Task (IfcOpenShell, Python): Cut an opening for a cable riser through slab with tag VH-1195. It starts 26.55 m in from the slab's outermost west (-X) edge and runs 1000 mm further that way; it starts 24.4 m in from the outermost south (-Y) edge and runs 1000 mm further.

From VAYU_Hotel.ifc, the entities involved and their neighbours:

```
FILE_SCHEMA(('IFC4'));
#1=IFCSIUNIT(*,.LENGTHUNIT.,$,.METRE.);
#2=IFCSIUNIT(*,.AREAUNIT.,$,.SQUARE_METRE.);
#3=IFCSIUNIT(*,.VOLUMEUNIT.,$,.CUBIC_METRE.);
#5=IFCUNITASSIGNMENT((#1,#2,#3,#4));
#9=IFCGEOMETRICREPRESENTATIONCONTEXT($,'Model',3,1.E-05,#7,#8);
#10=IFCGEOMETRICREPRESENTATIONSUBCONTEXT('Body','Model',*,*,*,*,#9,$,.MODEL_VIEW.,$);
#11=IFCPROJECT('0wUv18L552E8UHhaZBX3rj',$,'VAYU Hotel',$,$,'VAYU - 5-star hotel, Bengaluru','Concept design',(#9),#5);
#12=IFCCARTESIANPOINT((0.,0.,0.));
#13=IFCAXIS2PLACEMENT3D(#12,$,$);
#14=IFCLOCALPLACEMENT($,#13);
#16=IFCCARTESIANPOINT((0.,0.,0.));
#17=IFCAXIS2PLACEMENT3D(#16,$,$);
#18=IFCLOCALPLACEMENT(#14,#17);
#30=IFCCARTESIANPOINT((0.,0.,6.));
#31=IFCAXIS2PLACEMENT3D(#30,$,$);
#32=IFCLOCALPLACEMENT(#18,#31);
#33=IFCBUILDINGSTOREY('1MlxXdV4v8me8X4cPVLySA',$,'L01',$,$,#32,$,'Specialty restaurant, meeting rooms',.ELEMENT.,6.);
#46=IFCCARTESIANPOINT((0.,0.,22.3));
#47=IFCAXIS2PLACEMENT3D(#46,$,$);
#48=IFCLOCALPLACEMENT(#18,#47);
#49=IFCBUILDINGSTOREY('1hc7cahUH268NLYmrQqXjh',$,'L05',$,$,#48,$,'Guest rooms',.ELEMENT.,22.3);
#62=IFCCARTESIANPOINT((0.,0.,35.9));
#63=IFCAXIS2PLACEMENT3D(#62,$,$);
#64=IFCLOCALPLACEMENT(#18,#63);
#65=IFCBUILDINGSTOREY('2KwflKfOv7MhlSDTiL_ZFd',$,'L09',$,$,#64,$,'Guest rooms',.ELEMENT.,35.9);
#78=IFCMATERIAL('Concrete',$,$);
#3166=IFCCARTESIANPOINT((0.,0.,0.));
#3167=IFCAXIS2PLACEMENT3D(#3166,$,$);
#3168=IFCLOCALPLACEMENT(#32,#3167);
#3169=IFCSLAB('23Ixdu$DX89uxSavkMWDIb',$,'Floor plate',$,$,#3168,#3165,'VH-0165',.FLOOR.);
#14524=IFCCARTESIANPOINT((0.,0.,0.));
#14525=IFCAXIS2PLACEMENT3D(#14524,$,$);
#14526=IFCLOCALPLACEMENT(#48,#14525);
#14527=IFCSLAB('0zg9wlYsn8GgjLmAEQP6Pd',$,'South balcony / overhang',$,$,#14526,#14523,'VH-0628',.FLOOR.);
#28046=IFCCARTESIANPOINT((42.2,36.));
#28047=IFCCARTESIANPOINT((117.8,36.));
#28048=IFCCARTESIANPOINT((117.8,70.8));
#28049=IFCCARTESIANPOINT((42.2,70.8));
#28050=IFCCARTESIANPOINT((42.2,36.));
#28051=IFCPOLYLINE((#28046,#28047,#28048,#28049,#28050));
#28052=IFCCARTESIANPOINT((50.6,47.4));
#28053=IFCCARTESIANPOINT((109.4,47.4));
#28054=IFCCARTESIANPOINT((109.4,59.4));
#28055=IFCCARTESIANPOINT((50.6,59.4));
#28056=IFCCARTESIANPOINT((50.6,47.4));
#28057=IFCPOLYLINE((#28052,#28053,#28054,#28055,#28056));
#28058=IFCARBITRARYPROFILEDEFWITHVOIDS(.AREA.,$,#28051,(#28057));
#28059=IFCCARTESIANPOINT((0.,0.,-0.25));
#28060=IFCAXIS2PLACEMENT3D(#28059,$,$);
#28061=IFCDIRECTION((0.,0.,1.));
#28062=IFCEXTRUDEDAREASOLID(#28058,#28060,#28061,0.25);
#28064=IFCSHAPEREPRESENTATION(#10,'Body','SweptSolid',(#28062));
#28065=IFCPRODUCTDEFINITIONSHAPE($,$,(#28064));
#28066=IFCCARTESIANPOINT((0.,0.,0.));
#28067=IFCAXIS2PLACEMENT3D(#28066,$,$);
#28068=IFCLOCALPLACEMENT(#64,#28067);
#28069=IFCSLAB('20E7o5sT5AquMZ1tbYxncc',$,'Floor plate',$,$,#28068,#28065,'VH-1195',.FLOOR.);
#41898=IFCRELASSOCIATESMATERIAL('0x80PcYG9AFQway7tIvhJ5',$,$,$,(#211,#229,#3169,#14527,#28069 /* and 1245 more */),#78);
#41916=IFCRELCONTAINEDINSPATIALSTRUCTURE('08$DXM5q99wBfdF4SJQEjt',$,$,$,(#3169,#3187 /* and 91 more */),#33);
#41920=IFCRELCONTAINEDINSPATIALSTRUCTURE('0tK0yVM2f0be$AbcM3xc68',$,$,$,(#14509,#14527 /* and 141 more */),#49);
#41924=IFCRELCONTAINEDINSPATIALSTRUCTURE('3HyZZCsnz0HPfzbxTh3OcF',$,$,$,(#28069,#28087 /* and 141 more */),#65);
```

```python
import numpy as np
import ifcopenshell
import ifcopenshell.api.feature
import ifcopenshell.api.geometry
import ifcopenshell.api.root
import ifcopenshell.geom
import ifcopenshell.util.placement
import ifcopenshell.util.representation
import ifcopenshell.util.shape
import ifcopenshell.util.unit

model = ifcopenshell.open("VAYU_Hotel.ifc")
unit_scale = ifcopenshell.util.unit.calculate_unit_scale(model)
settings = ifcopenshell.geom.settings()


def volume(element):
    """Net volume in cubic metres, openings subtracted."""
    shape = ifcopenshell.geom.create_shape(settings, element)
    return ifcopenshell.util.shape.get_volume(shape.geometry)


slab = model.by_guid("20E7o5sT5AquMZ1tbYxncc")
before = volume(slab)

# Extent in the slab's own axes, in metres. The edges named are its -X and -Y sides.
slab_shape = ifcopenshell.geom.create_shape(settings, slab)
vertices = ifcopenshell.util.shape.get_vertices(slab_shape.geometry)
x_min, y_min, bottom = vertices.min(axis=0)
top = vertices[:, 2].max()

opening = ifcopenshell.api.root.create_entity(model, ifc_class="IfcOpeningElement", name="Cable riser opening", predefined_type="OPENING")
context = ifcopenshell.util.representation.get_context(model, "Model", "Body", "MODEL_VIEW")
width, depth = 1, 1
outline = [(0.0, 0.0), (width, 0.0), (width, depth), (0.0, depth), (0.0, 0.0)]
# Overshoot both faces by 50 mm so the cut is clean.
shape = ifcopenshell.api.geometry.add_slab_representation(
    model, context=context, depth=top - bottom + 0.1, polyline=outline
)
ifcopenshell.api.geometry.assign_representation(model, product=opening, representation=shape)

matrix = ifcopenshell.util.placement.get_local_placement(slab.ObjectPlacement)
matrix[:, 3] = matrix @ np.append(np.array([x_min + 26.55, y_min + 24.4, bottom - 0.05]) / unit_scale, 1.0)
ifcopenshell.api.geometry.edit_object_placement(model, product=opening, matrix=matrix, is_si=False)
ifcopenshell.api.feature.add_feature(model, feature=opening, element=slab)

after = volume(slab)

print(f"slab volume {before:.3f} -> {after:.3f} m3")

model.write("VAYU_Hotel_updated.ifc")
```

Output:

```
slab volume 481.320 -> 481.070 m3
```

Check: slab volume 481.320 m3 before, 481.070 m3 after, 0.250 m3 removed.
